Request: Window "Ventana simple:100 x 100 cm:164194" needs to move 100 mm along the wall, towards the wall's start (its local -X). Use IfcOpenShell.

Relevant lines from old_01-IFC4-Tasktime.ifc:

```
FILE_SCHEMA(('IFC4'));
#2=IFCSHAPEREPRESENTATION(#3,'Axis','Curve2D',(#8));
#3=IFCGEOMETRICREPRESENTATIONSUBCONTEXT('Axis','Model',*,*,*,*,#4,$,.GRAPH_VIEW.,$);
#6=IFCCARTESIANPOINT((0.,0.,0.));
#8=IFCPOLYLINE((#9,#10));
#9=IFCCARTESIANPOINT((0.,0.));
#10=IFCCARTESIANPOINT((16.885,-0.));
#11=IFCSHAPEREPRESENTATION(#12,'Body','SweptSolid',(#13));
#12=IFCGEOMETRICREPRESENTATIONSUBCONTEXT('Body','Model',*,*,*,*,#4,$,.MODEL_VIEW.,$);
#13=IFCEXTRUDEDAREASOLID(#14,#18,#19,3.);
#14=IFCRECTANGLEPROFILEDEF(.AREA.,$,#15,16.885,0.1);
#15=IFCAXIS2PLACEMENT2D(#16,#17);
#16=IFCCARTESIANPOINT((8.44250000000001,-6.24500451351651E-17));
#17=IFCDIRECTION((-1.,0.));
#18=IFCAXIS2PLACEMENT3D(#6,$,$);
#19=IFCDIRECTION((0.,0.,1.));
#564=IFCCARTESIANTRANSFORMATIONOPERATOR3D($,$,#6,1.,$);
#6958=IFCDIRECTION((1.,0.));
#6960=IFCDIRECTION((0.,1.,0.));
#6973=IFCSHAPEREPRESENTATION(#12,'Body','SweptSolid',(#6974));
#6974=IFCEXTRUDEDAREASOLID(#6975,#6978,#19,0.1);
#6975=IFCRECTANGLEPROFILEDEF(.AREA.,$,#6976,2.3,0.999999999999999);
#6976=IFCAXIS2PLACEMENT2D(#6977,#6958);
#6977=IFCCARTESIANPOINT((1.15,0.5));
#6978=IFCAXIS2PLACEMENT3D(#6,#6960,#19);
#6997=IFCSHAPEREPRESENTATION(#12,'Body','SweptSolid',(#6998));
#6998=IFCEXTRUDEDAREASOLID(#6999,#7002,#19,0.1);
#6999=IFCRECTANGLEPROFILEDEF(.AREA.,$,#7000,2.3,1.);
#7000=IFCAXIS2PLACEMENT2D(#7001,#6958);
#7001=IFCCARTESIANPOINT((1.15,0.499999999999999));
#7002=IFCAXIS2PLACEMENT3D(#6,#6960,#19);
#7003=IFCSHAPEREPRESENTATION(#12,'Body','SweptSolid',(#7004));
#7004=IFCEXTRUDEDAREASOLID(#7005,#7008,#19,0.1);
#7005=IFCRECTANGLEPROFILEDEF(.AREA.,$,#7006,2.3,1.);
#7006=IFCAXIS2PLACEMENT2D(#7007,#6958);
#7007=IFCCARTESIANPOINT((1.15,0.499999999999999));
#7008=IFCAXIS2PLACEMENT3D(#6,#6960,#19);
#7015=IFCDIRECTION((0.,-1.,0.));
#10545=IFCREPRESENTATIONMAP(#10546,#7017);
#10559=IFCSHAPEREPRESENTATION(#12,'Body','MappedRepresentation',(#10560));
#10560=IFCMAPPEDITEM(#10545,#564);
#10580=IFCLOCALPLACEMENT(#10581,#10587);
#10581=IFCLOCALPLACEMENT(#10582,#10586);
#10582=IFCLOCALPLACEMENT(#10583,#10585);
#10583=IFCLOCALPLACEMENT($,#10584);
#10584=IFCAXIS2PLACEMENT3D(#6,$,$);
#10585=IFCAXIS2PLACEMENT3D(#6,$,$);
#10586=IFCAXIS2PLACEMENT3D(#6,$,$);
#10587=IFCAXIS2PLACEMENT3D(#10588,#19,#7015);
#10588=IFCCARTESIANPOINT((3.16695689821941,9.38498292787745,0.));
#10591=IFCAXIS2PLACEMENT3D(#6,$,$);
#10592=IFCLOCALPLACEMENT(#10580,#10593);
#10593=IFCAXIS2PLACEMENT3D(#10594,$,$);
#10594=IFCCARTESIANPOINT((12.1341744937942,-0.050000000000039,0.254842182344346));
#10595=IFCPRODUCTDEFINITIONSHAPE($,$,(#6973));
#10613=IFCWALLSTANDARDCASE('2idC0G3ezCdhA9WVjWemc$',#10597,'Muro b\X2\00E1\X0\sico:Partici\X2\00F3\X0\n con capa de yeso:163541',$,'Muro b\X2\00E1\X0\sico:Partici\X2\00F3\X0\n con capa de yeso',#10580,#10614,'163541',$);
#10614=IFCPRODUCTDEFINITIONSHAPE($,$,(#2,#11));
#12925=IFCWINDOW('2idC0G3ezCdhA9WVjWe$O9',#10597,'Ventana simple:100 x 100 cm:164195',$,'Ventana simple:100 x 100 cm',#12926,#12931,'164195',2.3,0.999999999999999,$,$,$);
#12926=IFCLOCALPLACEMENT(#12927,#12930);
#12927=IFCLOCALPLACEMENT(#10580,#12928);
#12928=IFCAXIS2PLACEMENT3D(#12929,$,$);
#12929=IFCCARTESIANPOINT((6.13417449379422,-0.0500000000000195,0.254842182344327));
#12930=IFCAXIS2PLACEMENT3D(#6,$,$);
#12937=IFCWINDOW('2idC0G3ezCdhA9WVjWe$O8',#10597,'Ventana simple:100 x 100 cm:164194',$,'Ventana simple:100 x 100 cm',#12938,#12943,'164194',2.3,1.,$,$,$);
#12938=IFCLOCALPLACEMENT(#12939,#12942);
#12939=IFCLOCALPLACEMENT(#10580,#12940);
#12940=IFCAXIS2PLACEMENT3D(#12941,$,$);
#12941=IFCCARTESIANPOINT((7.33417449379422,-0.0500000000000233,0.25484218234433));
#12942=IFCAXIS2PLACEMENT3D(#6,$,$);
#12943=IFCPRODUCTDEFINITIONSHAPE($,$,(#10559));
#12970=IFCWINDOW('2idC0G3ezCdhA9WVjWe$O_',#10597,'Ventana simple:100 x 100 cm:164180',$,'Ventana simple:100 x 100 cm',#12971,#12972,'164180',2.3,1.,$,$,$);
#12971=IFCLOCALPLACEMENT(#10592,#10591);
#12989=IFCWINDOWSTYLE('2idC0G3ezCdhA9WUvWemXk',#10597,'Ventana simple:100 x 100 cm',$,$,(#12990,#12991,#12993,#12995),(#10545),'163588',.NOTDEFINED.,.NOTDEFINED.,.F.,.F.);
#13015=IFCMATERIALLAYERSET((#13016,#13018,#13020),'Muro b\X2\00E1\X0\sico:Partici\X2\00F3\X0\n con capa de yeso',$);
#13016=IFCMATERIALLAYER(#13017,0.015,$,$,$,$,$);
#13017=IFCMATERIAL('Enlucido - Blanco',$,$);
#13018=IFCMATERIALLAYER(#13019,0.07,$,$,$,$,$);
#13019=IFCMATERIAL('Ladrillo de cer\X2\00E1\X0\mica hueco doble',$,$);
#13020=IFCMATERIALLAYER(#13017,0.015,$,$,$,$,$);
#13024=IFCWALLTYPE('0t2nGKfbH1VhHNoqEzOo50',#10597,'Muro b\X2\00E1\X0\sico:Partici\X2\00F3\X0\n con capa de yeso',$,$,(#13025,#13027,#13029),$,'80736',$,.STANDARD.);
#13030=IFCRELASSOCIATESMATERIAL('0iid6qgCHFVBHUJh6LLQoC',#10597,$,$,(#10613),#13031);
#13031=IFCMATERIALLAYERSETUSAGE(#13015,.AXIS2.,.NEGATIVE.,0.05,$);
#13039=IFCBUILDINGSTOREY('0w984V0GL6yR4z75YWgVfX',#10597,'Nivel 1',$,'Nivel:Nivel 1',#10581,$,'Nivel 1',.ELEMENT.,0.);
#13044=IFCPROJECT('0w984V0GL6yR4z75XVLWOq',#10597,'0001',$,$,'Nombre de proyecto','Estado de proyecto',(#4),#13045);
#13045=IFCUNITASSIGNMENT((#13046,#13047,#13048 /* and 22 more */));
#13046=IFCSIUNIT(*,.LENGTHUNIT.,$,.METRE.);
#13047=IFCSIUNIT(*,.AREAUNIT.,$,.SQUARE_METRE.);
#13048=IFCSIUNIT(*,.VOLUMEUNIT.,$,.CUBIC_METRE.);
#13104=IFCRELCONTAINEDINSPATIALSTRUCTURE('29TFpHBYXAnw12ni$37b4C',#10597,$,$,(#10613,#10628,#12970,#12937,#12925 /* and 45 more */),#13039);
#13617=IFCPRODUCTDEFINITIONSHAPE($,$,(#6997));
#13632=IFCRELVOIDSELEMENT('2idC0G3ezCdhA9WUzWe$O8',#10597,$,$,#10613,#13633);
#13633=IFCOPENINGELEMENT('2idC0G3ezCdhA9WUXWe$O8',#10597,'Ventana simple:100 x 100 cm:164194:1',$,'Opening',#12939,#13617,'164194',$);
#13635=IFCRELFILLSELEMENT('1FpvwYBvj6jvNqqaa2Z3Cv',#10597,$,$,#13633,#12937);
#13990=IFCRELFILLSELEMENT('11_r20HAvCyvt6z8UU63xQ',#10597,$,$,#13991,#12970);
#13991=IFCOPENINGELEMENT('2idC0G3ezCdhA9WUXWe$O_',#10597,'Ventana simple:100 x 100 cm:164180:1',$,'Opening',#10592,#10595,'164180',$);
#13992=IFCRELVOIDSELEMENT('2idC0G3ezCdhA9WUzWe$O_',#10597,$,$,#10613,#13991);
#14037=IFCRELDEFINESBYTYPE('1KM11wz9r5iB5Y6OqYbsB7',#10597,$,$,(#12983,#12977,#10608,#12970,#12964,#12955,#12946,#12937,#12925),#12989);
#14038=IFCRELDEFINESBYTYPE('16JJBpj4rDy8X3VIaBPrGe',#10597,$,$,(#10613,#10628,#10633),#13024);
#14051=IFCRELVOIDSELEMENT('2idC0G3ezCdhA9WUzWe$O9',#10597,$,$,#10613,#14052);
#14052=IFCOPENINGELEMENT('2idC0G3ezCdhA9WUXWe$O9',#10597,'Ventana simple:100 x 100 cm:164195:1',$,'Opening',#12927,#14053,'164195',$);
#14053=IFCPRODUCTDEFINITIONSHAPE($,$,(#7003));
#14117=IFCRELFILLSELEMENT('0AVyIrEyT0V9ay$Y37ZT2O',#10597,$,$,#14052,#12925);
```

```python
import ifcopenshell
import ifcopenshell.api.geometry
import ifcopenshell.util.placement

model = ifcopenshell.open("old_01-IFC4-Tasktime.ifc")

window = model.by_guid("2idC0G3ezCdhA9WVjWe$O8")
opening = window.FillsVoids[0].RelatingOpeningElement
wall = opening.VoidsElements[0].RelatingBuildingElement

wall_matrix = ifcopenshell.util.placement.get_local_placement(wall.ObjectPlacement)
shift = wall_matrix[:3, 0] * -0.1
before = ifcopenshell.util.placement.get_local_placement(window.ObjectPlacement)[:3, 3].copy()

# The window is placed relative to its opening, so it follows when the opening moves.
matrix = ifcopenshell.util.placement.get_local_placement(opening.ObjectPlacement)
matrix[:3, 3] += shift
ifcopenshell.api.geometry.edit_object_placement(
    model, product=opening, matrix=matrix, is_si=False, should_transform_children=True
)

after = ifcopenshell.util.placement.get_local_placement(window.ObjectPlacement)[:3, 3]
print("window moved by", (after - before).round(3) + 0.0)

model.write("old_01-IFC4-Tasktime_rev.ifc")
```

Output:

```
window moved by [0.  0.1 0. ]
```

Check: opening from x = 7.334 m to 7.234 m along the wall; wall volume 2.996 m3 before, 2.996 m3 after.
